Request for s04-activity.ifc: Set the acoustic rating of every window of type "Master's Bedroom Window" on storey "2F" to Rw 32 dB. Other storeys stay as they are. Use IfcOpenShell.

First a look at what the model holds.

```python
import ifcopenshell
import ifcopenshell.util.element

model = ifcopenshell.open("s04-activity.ifc")
print(model.schema)
storey = next(s for s in model.by_type("IfcBuildingStorey") if s.Name == "2F")
windows = [e for e in ifcopenshell.util.element.get_decomposition(storey) if e.is_a("IfcWindow")]
seen = {}
for e in windows:
    element_type = ifcopenshell.util.element.get_type(e)
    key = (element_type.Name if element_type != e and element_type else None, ifcopenshell.util.element.get_pset(e, "Pset_WindowCommon", "AcousticRating"))
    seen[key] = seen.get(key, 0) + 1
for (name, value), count in sorted(seen.items(), key=str):
    print(count, "x", name, "|", value)
```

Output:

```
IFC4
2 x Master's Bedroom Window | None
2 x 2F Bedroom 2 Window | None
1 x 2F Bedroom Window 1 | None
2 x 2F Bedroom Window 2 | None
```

```python
import ifcopenshell
import ifcopenshell.api.pset
import ifcopenshell.util.element

model = ifcopenshell.open("s04-activity.ifc")

storey = next(s for s in model.by_type("IfcBuildingStorey") if s.Name == "2F")
windows = [e for e in ifcopenshell.util.element.get_decomposition(storey) if e.is_a("IfcWindow")]

count = 0
for e in windows:
    element_type = ifcopenshell.util.element.get_type(e)
    if element_type in (None, e) or element_type.Name != "Master's Bedroom Window":
        continue
    # add_pset returns the element's existing set when there is one.
    pset = ifcopenshell.api.pset.add_pset(model, product=e, name="Pset_WindowCommon")
    ifcopenshell.api.pset.edit_pset(model, pset=pset, properties={"AcousticRating": "Rw 32 dB"})
    count += 1

print(count, "windows updated")

model.write("s04-activity-out.ifc")
```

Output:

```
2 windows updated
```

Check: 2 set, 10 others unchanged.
